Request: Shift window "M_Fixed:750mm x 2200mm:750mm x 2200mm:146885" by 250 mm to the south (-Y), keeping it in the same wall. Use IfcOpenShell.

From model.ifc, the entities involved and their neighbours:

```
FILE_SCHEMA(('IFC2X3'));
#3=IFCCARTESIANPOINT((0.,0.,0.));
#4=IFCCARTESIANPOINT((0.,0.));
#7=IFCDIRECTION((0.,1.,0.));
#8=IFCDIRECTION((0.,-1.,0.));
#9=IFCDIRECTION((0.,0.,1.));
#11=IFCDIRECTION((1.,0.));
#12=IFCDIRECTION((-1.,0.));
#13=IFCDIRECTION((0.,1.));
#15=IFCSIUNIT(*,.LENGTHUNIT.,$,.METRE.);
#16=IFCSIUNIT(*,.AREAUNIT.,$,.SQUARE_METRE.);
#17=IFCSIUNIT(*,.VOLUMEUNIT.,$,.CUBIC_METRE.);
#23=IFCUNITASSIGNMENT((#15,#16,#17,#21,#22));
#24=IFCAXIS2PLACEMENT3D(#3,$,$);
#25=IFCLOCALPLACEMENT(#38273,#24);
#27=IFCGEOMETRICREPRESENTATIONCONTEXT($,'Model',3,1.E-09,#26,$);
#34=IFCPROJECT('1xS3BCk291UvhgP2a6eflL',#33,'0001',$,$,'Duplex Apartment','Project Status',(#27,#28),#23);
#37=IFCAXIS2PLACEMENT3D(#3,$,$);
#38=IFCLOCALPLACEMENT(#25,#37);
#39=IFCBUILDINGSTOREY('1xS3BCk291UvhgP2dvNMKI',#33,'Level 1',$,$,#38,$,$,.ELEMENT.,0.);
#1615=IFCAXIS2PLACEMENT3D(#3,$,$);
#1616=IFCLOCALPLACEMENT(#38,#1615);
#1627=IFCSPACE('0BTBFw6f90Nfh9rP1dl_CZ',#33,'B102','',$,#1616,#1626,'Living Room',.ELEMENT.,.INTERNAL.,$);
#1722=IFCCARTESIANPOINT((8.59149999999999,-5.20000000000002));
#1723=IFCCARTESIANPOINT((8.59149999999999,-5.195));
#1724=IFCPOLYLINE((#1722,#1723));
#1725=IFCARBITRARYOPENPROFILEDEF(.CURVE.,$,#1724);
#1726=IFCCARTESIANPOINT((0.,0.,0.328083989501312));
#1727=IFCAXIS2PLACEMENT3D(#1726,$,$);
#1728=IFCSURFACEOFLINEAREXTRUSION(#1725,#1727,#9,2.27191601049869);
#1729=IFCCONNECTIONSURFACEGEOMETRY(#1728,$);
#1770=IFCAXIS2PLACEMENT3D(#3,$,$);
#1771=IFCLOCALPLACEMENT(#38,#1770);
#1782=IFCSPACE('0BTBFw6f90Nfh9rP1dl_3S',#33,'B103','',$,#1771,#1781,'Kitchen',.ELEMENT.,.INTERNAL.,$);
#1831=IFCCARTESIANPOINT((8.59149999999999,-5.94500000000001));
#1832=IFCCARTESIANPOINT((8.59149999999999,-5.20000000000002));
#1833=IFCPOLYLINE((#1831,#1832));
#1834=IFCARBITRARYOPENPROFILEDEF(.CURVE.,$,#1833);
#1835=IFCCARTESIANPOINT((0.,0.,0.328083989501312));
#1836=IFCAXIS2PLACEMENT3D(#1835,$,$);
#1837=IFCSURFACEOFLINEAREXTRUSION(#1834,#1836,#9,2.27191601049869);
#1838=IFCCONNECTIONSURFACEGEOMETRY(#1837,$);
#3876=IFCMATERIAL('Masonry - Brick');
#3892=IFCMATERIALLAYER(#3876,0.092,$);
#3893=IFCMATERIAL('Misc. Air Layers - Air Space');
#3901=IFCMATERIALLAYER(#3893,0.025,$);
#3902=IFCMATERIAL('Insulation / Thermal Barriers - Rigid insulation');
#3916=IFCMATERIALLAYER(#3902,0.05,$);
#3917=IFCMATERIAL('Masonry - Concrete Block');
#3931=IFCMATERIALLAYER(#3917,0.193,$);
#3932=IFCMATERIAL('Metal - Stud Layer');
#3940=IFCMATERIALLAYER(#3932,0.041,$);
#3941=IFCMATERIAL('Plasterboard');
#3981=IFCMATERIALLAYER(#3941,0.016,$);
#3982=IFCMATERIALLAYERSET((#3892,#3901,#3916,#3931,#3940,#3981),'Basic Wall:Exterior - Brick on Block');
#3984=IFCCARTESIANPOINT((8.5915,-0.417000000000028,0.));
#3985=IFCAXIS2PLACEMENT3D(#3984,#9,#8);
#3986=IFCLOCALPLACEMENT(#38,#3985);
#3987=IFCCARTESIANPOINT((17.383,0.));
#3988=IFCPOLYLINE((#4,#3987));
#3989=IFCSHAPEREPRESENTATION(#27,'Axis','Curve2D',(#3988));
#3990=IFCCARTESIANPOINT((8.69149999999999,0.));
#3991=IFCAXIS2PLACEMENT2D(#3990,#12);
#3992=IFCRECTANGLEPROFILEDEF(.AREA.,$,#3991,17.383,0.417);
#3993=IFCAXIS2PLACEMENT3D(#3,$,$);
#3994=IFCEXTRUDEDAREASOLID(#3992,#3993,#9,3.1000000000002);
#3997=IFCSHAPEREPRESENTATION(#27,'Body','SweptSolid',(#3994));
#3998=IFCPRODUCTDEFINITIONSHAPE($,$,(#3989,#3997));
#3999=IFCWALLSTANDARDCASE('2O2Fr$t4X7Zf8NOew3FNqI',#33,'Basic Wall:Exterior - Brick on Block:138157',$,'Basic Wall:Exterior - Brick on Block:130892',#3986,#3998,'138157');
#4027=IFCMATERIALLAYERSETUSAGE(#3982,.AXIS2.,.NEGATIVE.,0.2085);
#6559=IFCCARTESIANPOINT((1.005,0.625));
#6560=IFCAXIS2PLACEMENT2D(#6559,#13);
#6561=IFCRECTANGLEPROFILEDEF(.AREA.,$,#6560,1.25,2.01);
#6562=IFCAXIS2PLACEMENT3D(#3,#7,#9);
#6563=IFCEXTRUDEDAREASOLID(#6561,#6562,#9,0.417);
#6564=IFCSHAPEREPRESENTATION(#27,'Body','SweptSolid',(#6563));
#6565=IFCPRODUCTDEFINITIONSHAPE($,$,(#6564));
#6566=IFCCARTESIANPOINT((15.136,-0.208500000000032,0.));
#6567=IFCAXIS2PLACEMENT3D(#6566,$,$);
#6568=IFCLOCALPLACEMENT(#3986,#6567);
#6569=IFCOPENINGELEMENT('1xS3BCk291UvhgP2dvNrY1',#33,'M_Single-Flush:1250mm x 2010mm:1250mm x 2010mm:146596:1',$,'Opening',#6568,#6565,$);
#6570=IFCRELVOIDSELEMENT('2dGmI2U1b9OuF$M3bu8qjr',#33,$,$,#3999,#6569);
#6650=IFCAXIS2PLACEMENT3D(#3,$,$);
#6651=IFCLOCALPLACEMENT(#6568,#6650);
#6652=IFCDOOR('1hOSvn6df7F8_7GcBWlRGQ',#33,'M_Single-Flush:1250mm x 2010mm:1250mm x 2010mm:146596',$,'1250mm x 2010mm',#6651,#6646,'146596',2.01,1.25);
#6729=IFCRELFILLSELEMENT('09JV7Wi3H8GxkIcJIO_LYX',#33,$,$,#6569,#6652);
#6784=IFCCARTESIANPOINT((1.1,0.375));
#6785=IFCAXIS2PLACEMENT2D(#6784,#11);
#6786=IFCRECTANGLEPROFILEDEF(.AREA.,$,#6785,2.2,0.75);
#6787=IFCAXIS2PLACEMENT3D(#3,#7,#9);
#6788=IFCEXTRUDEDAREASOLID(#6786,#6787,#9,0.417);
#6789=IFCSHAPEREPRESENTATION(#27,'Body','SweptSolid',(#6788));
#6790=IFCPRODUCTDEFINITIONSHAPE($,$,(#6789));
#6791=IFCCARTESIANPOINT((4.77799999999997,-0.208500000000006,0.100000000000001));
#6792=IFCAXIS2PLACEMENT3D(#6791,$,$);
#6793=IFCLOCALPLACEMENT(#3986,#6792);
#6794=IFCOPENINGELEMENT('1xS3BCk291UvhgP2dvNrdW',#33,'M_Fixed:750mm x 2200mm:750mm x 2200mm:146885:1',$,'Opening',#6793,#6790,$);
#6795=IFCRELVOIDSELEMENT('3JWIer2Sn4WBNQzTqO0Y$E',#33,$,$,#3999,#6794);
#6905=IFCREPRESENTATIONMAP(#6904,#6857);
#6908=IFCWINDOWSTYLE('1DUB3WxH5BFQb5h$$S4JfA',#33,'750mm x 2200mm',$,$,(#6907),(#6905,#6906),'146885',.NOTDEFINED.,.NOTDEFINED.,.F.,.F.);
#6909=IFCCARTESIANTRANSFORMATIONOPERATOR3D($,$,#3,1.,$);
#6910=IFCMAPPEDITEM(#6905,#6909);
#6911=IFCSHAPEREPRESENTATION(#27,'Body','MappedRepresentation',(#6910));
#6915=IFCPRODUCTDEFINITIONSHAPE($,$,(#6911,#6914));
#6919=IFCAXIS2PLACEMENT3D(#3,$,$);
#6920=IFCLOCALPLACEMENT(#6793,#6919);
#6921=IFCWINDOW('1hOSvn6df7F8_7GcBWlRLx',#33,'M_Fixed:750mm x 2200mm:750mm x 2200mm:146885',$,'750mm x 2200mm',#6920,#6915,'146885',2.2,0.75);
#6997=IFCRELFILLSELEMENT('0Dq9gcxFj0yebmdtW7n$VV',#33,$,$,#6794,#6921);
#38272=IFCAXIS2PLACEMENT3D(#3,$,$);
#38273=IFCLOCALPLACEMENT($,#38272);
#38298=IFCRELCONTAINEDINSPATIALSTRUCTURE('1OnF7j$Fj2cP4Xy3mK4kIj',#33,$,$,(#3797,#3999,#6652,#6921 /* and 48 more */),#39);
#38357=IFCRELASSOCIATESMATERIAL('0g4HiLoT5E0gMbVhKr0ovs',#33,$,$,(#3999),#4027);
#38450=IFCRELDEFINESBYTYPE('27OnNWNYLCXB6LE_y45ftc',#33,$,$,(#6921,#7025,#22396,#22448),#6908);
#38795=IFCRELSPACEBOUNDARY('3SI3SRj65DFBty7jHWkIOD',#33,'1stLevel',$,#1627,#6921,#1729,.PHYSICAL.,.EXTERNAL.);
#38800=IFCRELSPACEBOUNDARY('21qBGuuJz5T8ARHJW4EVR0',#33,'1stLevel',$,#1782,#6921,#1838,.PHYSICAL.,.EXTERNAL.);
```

```python
import numpy as np
import ifcopenshell
import ifcopenshell.api.geometry
import ifcopenshell.util.placement
import ifcopenshell.util.unit

model = ifcopenshell.open("model.ifc")
unit_scale = ifcopenshell.util.unit.calculate_unit_scale(model)

window = model.by_guid("1hOSvn6df7F8_7GcBWlRLx")
opening = window.FillsVoids[0].RelatingOpeningElement
wall = opening.VoidsElements[0].RelatingBuildingElement

wall_matrix = ifcopenshell.util.placement.get_local_placement(wall.ObjectPlacement)
shift = wall_matrix[:3, 0] * 0.25 / unit_scale
before = ifcopenshell.util.placement.get_local_placement(window.ObjectPlacement)[:3, 3].copy()

# The window is placed relative to its opening, so it follows when the opening moves.
matrix = ifcopenshell.util.placement.get_local_placement(opening.ObjectPlacement)
matrix[:3, 3] += shift
ifcopenshell.api.geometry.edit_object_placement(
    model, product=opening, matrix=matrix, is_si=False, should_transform_children=True
)

# Space boundary surfaces are stored in each space's coordinates; move them too.
for rel in window.ProvidesBoundaries:
    if not rel.ConnectionGeometry:
        continue
    surface = rel.ConnectionGeometry.SurfaceOnRelatingElement
    space_matrix = ifcopenshell.util.placement.get_local_placement(rel.RelatingSpace.ObjectPlacement)
    point = np.array(surface.Position.Location.Coordinates) + space_matrix[:3, :3].T @ shift
    surface.Position = model.createIfcAxis2Placement3D(
        model.createIfcCartesianPoint(point.tolist()), surface.Position.Axis, surface.Position.RefDirection
    )

after = ifcopenshell.util.placement.get_local_placement(window.ObjectPlacement)[:3, 3]
print("window moved by", (after - before).round(3) + 0.0)

model.write("model_edited.ifc")
```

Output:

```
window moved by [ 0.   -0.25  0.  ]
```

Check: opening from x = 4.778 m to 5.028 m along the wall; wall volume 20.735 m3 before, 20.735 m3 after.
